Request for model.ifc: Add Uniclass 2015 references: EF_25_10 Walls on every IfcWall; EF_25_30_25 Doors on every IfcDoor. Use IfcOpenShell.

First a look at what the model holds.

```python
import ifcopenshell

model = ifcopenshell.open("model.ifc")
print(model.schema)
print("classifications:", [c.Name for c in model.by_type("IfcClassification")])
for ifc_class in ("IfcDoor", "IfcRoof", "IfcStair", "IfcWall", "IfcWindow"):
    print(ifc_class, len(model.by_type(ifc_class)))
```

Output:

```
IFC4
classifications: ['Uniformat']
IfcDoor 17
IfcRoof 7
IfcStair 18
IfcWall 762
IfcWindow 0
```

```python
import ifcopenshell
import ifcopenshell.api.classification

model = ifcopenshell.open("model.ifc")

system = ifcopenshell.api.classification.add_classification(model, classification="Uniclass 2015")

codes = {
    "IfcWall": ("EF_25_10", "Walls"),
    "IfcDoor": ("EF_25_30_25", "Doors"),
}
for ifc_class, (code, name) in codes.items():
    products = model.by_type(ifc_class)
    ifcopenshell.api.classification.add_reference(
        model, products=products, classification=system, identification=code, name=name
    )
    print(code, len(products))

model.write("model_rev.ifc")
```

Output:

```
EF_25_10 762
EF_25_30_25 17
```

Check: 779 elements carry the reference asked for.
